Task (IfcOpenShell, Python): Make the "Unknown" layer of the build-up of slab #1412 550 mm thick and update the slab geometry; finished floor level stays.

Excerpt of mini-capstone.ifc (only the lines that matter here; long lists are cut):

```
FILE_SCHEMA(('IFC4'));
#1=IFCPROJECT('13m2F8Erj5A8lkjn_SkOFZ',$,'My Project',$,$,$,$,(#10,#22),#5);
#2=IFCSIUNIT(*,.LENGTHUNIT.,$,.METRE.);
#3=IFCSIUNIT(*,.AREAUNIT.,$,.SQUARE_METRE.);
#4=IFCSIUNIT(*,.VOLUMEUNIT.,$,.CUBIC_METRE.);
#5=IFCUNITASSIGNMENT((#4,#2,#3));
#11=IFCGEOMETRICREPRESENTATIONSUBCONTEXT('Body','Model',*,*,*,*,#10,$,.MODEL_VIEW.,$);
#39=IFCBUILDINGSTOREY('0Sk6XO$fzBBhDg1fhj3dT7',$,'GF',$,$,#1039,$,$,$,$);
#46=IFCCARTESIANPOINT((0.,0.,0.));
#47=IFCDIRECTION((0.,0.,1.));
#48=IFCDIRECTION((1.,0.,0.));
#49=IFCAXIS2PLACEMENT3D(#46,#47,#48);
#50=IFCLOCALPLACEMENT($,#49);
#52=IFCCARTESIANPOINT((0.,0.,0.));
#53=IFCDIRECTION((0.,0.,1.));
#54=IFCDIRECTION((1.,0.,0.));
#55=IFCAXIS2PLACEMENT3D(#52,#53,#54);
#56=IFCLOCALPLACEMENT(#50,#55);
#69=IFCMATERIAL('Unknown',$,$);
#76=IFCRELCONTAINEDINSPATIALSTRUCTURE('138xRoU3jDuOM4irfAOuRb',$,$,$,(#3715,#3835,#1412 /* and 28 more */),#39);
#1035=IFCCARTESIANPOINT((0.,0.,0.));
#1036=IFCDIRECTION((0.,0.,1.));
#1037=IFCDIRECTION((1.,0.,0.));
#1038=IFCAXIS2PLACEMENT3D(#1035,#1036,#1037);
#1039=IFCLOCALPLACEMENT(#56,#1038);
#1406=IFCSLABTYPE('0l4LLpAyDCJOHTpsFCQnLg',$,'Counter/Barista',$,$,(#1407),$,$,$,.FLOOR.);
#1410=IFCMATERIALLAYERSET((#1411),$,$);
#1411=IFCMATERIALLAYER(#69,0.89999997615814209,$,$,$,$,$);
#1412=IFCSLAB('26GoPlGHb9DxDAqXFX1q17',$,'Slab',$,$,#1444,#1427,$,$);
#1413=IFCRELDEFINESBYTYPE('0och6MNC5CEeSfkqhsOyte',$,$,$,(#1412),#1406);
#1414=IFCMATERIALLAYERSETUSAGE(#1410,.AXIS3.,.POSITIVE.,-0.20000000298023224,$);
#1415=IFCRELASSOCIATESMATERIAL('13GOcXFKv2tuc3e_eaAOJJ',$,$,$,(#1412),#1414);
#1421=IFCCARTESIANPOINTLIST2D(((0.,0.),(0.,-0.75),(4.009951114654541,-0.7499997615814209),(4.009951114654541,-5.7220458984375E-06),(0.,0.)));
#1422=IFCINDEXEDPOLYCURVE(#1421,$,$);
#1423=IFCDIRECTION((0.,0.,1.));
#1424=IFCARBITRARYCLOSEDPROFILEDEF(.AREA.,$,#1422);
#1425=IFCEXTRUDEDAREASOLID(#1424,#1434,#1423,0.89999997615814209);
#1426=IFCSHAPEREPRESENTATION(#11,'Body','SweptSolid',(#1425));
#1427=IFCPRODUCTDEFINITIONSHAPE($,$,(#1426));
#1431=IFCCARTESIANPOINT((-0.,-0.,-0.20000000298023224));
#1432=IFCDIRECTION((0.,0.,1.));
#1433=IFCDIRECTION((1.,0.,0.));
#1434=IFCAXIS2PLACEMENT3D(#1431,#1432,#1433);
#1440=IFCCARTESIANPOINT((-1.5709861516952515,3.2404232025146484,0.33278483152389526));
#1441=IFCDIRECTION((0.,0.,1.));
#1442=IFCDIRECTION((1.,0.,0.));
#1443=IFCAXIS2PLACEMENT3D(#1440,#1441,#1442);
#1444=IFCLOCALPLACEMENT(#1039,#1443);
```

```python
import ifcopenshell
import ifcopenshell.util.element
import ifcopenshell.util.representation
import ifcopenshell.util.unit

model = ifcopenshell.open("mini-capstone.ifc")
unit_scale = ifcopenshell.util.unit.calculate_unit_scale(model)

layer_set = model.by_id(1410)
layer = next(l for l in layer_set.MaterialLayers if l.Material and l.Material.Name == "Unknown")
change = 0.55 / unit_scale - layer.LayerThickness
layer.LayerThickness += change

# Geometry does not follow the layer set by itself.
slabs = [e for e in ifcopenshell.util.element.get_elements_by_material(model, layer_set) if e.is_a("IfcSlab")]
for slab in sorted(slabs, key=lambda e: e.id()):
    body = ifcopenshell.util.representation.get_representation(slab, "Model", "Body")
    solid = body.Items[0]
    old_depth = solid.Depth
    solid.Depth += change
    # Extruded upwards: lower the start of the extrusion so the top stays.
    x, y, z = solid.Position.Location.Coordinates
    solid.Position.Location = model.createIfcCartesianPoint((x, y, z - change))
    print(slab.id(), f"{old_depth:g} -> {solid.Depth:g}")

# The layers are counted up from the underside, which has moved.
for usage in {ifcopenshell.util.element.get_material(slab) for slab in slabs}:
    usage.OffsetFromReferenceLine -= change

model.write("mini-capstone_rev.ifc")
```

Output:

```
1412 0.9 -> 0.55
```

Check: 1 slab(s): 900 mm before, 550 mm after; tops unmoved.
